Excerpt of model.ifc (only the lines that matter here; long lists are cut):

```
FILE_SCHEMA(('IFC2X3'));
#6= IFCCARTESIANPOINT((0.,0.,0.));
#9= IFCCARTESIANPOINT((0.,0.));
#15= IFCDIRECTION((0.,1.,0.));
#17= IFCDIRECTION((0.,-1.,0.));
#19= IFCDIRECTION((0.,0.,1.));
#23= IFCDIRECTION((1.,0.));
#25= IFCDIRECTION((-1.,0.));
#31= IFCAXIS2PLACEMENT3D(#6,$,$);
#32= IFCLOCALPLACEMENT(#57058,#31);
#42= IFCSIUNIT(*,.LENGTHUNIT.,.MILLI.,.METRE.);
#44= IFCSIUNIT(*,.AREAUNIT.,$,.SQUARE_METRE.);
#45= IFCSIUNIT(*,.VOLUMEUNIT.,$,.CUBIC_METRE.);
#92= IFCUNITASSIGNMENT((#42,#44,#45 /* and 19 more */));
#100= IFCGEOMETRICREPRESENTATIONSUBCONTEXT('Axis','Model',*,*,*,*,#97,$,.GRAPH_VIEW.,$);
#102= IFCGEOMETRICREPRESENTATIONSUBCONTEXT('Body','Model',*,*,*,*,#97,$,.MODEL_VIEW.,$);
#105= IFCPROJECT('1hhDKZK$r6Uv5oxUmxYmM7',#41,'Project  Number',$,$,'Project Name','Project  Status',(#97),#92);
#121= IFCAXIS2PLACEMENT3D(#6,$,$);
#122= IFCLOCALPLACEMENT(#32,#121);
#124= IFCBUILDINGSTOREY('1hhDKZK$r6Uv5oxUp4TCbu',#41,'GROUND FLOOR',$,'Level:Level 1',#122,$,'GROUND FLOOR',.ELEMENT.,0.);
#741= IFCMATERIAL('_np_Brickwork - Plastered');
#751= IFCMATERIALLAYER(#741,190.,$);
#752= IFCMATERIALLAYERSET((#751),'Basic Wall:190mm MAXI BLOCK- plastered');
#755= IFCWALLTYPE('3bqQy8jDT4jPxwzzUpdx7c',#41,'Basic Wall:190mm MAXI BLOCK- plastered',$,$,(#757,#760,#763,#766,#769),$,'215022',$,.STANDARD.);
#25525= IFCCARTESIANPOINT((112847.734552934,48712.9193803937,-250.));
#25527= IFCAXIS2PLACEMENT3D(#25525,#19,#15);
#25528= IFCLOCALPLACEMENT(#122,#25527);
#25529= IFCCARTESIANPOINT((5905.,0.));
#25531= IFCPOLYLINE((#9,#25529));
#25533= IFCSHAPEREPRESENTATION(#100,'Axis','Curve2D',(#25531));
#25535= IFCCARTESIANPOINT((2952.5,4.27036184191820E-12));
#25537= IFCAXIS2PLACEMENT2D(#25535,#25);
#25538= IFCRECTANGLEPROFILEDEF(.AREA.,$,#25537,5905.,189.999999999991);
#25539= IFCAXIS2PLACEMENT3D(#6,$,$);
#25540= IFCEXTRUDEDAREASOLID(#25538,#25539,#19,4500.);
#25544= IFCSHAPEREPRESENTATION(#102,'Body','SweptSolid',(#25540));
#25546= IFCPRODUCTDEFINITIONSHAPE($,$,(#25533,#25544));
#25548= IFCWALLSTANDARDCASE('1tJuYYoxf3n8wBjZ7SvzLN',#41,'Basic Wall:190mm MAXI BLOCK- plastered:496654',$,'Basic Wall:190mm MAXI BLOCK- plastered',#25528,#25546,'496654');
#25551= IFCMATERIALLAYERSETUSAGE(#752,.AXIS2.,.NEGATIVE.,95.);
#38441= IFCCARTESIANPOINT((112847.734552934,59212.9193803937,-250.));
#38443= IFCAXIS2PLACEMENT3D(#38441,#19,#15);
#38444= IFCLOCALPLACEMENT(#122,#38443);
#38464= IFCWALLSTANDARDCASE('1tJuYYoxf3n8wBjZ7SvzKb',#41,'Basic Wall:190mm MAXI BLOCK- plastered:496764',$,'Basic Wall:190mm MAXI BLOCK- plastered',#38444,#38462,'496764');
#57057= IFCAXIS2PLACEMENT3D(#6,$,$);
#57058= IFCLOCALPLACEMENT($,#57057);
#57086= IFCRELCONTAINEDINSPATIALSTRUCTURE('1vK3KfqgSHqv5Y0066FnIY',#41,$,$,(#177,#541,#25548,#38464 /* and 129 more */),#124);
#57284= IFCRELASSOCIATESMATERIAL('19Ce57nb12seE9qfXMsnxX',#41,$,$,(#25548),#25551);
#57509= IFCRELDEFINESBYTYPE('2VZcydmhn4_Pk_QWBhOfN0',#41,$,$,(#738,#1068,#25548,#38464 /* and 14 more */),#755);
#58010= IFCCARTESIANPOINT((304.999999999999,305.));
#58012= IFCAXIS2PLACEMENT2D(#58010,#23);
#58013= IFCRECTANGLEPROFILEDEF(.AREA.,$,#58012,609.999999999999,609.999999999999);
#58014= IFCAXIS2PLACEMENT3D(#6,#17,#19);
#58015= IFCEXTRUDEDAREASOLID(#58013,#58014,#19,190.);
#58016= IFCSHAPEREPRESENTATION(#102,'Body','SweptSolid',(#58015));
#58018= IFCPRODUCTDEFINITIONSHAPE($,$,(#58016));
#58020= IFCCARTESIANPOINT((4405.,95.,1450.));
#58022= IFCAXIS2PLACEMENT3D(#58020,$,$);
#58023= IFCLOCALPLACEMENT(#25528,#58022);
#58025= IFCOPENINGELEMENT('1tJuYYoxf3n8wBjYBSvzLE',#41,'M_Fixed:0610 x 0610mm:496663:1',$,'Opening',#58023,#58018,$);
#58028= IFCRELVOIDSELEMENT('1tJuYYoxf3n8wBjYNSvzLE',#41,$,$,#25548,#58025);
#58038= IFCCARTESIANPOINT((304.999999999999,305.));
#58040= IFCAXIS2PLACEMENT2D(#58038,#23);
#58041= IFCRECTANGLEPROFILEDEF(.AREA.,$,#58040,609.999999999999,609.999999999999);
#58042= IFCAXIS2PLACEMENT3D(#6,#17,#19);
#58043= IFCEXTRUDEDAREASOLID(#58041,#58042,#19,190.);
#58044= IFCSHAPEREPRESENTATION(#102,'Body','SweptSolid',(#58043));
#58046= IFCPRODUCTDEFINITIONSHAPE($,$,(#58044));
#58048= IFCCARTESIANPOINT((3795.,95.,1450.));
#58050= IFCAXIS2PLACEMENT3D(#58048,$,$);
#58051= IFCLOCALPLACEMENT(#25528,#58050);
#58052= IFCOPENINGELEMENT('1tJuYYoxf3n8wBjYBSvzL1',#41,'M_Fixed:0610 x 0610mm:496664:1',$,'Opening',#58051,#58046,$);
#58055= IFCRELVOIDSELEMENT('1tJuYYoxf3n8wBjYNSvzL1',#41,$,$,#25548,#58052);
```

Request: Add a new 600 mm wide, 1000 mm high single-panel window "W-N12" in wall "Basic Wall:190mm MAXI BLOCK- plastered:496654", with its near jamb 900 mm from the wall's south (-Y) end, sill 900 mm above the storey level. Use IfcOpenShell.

```python
import numpy as np
import ifcopenshell
import ifcopenshell.api.feature
import ifcopenshell.api.geometry
import ifcopenshell.api.root
import ifcopenshell.api.spatial
import ifcopenshell.api.type
import ifcopenshell.geom
import ifcopenshell.util.element
import ifcopenshell.util.placement
import ifcopenshell.util.representation
import ifcopenshell.util.shape
import ifcopenshell.util.unit

model = ifcopenshell.open("model.ifc")
unit_scale = ifcopenshell.util.unit.calculate_unit_scale(model)
settings = ifcopenshell.geom.settings()


def volume(element):
    """Net volume in cubic metres, openings subtracted."""
    shape = ifcopenshell.geom.create_shape(settings, element)
    return ifcopenshell.util.shape.get_volume(shape.geometry)


wall = model.by_guid("1tJuYYoxf3n8wBjZ7SvzLN")
storey = ifcopenshell.util.element.get_container(wall, ifc_class="IfcBuildingStorey")
context = ifcopenshell.util.representation.get_context(model, "Model", "Body", "MODEL_VIEW")
before = volume(wall)

width, height, from_end, sill = 0.6, 1, 0.9, 0.9  # metres

# The wall runs along its own X axis, and the end named is its -X end.
wall_shape = ifcopenshell.geom.create_shape(settings, wall)
x, y, z = ifcopenshell.util.shape.get_vertices(wall_shape.geometry).T
start = x.min() + from_end
face, thickness = float(y.min()), float(y.max() - y.min())
wall_matrix = ifcopenshell.util.placement.get_local_placement(wall.ObjectPlacement)
level = ifcopenshell.util.placement.get_local_placement(storey.ObjectPlacement)[2, 3]


def in_wall(x, y):
    """Placement at x, y metres in the wall's axes, at sill height."""
    matrix = wall_matrix.copy()
    matrix[:, 3] = wall_matrix @ np.array([x / unit_scale, y / unit_scale, 0.0, 1.0])
    matrix[2, 3] = level + sill / unit_scale
    return matrix


# Opening: a box that overshoots both wall faces by 50 mm.
opening = ifcopenshell.api.root.create_entity(model, ifc_class="IfcOpeningElement")
box = ifcopenshell.api.geometry.add_wall_representation(
    model, context=context, length=width, height=height, thickness=thickness + 0.1
)
ifcopenshell.api.geometry.assign_representation(model, product=opening, representation=box)
ifcopenshell.api.geometry.edit_object_placement(model, product=opening, matrix=in_wall(start, face - 0.05), is_si=False)
ifcopenshell.api.feature.add_feature(model, feature=opening, element=wall)

window = ifcopenshell.api.root.create_entity(model, ifc_class="IfcWindow", name="W-N12")
window.OverallWidth, window.OverallHeight = width / unit_scale, height / unit_scale
body = ifcopenshell.api.geometry.add_window_representation(
    model,
    context=context,
    overall_width=window.OverallWidth,
    overall_height=window.OverallHeight,
    partition_type="SINGLE_PANEL",
)
ifcopenshell.api.geometry.assign_representation(model, product=window, representation=body)
ifcopenshell.api.spatial.assign_container(model, products=[window], relating_structure=storey)
fills = ifcopenshell.api.feature.add_filling(model, opening=opening, element=window)
fills.OwnerHistory = window.OwnerHistory  # required in IFC2X3

# IFC2X3 keeps the operation on the window style.
style = ifcopenshell.api.root.create_entity(model, ifc_class="IfcWindowStyle", name="W-N12")
style.OperationType, style.ConstructionType = "SINGLE_PANEL", "NOTDEFINED"
style.ParameterTakesPrecedence = style.Sizeable = False
ifcopenshell.api.type.assign_type(model, related_objects=[window], relating_type=style)

# Centre the window in the wall's thickness.
ifcopenshell.api.geometry.edit_object_placement(model, product=window, matrix=in_wall(start, face), is_si=False)
window_shape = ifcopenshell.geom.create_shape(settings, window)
depth = ifcopenshell.util.shape.get_vertices(window_shape.geometry)[:, 1]
offset = face + thickness / 2 - (depth.min() + depth.max()) / 2
ifcopenshell.api.geometry.edit_object_placement(model, product=window, matrix=in_wall(start, offset), is_si=False)

after = volume(wall)

print(f"wall volume {before:.3f} -> {after:.3f} m3")

model.write("model_updated.ifc")
```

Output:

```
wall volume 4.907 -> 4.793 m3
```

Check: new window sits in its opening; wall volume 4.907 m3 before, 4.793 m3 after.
